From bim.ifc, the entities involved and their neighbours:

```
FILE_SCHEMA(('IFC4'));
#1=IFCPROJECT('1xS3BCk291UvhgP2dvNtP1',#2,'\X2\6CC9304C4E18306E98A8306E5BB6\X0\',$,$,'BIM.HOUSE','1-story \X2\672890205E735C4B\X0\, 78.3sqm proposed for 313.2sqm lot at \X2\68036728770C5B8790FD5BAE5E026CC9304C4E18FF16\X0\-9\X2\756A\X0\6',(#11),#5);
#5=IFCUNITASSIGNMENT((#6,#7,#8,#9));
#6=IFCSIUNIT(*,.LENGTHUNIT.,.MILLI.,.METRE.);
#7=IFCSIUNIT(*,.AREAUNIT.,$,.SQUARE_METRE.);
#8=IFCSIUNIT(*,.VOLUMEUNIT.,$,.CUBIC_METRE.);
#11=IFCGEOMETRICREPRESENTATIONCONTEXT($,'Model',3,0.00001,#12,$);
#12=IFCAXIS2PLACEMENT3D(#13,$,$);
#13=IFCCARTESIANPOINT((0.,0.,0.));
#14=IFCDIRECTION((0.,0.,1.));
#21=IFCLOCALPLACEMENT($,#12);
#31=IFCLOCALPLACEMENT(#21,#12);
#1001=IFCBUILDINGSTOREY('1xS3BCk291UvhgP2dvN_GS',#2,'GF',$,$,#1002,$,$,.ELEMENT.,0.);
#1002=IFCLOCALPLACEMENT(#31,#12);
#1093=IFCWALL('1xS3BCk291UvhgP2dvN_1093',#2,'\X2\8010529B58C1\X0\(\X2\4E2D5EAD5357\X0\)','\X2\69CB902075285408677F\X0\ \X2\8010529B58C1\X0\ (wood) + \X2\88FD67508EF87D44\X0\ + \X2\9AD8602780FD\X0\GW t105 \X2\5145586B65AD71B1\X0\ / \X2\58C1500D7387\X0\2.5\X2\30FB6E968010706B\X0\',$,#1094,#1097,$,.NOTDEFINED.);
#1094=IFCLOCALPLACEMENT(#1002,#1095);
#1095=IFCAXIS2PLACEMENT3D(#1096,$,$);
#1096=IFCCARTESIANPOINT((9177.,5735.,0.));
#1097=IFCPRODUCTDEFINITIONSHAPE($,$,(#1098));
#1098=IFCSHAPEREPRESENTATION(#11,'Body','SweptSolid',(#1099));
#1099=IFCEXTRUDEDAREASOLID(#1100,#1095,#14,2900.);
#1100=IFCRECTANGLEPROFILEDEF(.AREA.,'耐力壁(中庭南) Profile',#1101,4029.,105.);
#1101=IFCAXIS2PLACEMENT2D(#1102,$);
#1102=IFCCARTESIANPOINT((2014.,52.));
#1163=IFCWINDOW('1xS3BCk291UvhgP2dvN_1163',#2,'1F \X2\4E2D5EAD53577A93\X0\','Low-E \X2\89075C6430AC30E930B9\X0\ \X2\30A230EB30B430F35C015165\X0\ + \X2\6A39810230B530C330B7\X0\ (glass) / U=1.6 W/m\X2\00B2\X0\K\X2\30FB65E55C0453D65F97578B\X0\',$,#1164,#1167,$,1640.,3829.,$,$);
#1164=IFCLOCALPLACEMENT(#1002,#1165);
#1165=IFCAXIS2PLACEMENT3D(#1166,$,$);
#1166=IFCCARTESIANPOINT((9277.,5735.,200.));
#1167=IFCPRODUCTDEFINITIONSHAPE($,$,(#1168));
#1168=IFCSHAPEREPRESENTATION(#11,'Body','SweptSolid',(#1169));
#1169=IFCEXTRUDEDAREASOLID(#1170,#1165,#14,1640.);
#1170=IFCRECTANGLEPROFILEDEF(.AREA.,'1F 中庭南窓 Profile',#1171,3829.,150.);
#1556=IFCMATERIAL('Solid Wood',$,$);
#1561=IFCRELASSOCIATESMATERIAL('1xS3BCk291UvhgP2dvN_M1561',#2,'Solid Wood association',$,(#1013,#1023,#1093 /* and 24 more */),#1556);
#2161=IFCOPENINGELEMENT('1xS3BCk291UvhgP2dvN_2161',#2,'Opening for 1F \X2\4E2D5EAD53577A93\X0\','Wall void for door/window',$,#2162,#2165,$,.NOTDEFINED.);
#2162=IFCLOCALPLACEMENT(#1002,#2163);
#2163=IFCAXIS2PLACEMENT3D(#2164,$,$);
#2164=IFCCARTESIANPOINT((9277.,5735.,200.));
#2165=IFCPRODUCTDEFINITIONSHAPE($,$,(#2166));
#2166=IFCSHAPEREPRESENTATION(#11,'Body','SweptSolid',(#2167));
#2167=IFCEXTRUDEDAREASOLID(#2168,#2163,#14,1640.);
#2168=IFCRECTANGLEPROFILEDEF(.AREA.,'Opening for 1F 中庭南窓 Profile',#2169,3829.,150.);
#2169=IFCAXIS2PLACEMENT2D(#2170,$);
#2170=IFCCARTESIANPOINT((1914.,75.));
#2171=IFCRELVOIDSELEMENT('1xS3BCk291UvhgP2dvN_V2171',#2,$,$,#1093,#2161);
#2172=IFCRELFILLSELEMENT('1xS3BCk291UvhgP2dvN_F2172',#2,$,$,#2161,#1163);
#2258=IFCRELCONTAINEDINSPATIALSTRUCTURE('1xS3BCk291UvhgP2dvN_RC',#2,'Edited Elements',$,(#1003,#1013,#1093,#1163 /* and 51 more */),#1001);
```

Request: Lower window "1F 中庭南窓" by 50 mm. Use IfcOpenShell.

```python
import numpy as np
import ifcopenshell
import ifcopenshell.api.geometry
import ifcopenshell.util.placement
import ifcopenshell.util.unit

model = ifcopenshell.open("bim.ifc")
unit_scale = ifcopenshell.util.unit.calculate_unit_scale(model)

window = model.by_guid("1xS3BCk291UvhgP2dvN_1163")
opening = window.FillsVoids[0].RelatingOpeningElement
dz = -0.05 / unit_scale

shift = np.array([0.0, 0.0, dz])
# The window is not placed relative to its opening, so move both.
for product in (opening, window):
    matrix = ifcopenshell.util.placement.get_local_placement(product.ObjectPlacement)
    matrix[:3, 3] += shift
    ifcopenshell.api.geometry.edit_object_placement(model, product=product, matrix=matrix, is_si=False)

print(f"moved by {dz * unit_scale:+.3f} m")

model.write("bim_edited.ifc")
```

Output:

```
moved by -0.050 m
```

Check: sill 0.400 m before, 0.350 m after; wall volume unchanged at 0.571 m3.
